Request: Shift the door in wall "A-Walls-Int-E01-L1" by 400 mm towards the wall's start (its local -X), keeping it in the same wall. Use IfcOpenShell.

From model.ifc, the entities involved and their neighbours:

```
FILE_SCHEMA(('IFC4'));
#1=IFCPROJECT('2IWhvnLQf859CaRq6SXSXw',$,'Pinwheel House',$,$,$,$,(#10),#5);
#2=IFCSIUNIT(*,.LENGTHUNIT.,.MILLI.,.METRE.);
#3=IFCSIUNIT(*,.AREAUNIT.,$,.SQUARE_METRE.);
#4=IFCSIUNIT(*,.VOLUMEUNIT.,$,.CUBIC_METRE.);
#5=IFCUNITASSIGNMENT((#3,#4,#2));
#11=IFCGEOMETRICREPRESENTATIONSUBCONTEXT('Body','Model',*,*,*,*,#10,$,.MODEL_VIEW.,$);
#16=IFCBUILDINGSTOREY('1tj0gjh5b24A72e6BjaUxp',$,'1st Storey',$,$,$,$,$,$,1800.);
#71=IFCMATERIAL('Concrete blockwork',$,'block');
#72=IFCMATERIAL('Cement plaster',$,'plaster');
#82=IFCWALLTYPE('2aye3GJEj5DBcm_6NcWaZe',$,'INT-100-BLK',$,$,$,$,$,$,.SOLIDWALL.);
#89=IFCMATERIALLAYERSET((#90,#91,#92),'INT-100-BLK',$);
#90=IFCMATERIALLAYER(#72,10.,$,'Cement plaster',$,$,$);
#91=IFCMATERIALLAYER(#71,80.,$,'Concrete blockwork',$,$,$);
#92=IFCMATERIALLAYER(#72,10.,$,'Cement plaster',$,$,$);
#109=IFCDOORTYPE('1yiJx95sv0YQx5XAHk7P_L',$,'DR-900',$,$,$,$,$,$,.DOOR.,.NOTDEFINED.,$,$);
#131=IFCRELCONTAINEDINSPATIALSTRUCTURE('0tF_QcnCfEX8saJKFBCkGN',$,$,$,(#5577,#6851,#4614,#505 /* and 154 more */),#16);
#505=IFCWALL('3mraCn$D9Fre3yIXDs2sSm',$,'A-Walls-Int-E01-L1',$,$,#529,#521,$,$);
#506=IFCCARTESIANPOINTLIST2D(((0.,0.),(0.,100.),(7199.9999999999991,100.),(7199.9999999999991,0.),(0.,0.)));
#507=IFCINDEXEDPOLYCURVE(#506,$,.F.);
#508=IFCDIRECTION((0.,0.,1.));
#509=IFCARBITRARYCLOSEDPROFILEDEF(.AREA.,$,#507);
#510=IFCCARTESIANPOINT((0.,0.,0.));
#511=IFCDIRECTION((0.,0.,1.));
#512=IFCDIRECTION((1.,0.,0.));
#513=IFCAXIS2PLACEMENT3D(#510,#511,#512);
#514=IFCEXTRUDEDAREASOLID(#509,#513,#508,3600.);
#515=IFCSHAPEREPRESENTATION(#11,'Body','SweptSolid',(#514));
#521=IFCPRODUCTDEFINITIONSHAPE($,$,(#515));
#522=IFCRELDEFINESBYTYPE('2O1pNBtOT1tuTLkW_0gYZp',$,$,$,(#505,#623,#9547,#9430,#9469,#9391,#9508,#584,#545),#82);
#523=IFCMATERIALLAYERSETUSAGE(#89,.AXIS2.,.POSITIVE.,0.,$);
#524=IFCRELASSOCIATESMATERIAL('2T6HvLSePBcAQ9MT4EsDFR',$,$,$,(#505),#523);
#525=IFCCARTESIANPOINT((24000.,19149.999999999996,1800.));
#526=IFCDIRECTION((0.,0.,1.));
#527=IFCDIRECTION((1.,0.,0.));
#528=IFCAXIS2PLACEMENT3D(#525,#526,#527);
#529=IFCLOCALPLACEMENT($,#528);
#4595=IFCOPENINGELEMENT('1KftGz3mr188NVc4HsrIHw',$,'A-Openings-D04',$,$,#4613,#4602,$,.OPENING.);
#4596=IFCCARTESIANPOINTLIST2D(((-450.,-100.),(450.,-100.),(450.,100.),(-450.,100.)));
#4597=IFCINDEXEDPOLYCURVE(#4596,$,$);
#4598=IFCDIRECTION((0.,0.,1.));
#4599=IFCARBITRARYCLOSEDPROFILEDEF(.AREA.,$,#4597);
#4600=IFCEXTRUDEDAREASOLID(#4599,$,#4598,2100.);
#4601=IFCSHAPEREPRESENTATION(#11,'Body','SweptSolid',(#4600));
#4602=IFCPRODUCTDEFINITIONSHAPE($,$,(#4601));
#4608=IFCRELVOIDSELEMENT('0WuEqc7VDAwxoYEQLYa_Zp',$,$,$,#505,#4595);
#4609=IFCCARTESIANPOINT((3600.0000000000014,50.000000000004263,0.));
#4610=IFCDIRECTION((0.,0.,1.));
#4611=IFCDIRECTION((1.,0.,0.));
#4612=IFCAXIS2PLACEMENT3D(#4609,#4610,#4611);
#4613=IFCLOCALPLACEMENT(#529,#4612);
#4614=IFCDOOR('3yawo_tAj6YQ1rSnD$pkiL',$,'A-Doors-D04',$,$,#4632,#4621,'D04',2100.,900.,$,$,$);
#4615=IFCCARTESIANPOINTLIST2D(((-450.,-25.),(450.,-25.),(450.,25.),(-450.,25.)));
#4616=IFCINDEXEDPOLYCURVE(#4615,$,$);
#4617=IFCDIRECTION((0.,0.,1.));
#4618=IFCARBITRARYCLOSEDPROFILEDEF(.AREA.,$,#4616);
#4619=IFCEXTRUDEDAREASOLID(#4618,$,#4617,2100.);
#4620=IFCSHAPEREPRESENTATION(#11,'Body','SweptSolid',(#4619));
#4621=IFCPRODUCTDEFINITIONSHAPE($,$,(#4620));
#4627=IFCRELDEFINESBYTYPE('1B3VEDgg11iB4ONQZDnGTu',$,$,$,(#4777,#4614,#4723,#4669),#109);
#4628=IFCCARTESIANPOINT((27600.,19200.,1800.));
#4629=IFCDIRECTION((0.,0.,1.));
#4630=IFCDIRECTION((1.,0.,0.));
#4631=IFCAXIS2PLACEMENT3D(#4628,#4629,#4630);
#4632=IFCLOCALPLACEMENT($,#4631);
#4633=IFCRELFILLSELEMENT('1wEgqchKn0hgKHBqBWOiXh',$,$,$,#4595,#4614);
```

```python
import ifcopenshell
import ifcopenshell.api.geometry
import ifcopenshell.util.placement

model = ifcopenshell.open("model.ifc")

door = model.by_id(4614)
opening = door.FillsVoids[0].RelatingOpeningElement
wall = opening.VoidsElements[0].RelatingBuildingElement

wall_matrix = ifcopenshell.util.placement.get_local_placement(wall.ObjectPlacement)
shift = wall_matrix[:3, 0] * -400.0
before = ifcopenshell.util.placement.get_local_placement(door.ObjectPlacement)[:3, 3].copy()

# The door is not placed relative to its opening, so move both.
for product in (opening, door):
    matrix = ifcopenshell.util.placement.get_local_placement(product.ObjectPlacement)
    matrix[:3, 3] += shift
    ifcopenshell.api.geometry.edit_object_placement(model, product=product, matrix=matrix, is_si=False)

after = ifcopenshell.util.placement.get_local_placement(door.ObjectPlacement)[:3, 3]
print("door moved by", (after - before).round(3) + 0.0)

model.write("model-out.ifc")
```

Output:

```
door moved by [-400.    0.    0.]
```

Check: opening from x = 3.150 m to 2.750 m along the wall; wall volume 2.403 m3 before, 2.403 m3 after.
